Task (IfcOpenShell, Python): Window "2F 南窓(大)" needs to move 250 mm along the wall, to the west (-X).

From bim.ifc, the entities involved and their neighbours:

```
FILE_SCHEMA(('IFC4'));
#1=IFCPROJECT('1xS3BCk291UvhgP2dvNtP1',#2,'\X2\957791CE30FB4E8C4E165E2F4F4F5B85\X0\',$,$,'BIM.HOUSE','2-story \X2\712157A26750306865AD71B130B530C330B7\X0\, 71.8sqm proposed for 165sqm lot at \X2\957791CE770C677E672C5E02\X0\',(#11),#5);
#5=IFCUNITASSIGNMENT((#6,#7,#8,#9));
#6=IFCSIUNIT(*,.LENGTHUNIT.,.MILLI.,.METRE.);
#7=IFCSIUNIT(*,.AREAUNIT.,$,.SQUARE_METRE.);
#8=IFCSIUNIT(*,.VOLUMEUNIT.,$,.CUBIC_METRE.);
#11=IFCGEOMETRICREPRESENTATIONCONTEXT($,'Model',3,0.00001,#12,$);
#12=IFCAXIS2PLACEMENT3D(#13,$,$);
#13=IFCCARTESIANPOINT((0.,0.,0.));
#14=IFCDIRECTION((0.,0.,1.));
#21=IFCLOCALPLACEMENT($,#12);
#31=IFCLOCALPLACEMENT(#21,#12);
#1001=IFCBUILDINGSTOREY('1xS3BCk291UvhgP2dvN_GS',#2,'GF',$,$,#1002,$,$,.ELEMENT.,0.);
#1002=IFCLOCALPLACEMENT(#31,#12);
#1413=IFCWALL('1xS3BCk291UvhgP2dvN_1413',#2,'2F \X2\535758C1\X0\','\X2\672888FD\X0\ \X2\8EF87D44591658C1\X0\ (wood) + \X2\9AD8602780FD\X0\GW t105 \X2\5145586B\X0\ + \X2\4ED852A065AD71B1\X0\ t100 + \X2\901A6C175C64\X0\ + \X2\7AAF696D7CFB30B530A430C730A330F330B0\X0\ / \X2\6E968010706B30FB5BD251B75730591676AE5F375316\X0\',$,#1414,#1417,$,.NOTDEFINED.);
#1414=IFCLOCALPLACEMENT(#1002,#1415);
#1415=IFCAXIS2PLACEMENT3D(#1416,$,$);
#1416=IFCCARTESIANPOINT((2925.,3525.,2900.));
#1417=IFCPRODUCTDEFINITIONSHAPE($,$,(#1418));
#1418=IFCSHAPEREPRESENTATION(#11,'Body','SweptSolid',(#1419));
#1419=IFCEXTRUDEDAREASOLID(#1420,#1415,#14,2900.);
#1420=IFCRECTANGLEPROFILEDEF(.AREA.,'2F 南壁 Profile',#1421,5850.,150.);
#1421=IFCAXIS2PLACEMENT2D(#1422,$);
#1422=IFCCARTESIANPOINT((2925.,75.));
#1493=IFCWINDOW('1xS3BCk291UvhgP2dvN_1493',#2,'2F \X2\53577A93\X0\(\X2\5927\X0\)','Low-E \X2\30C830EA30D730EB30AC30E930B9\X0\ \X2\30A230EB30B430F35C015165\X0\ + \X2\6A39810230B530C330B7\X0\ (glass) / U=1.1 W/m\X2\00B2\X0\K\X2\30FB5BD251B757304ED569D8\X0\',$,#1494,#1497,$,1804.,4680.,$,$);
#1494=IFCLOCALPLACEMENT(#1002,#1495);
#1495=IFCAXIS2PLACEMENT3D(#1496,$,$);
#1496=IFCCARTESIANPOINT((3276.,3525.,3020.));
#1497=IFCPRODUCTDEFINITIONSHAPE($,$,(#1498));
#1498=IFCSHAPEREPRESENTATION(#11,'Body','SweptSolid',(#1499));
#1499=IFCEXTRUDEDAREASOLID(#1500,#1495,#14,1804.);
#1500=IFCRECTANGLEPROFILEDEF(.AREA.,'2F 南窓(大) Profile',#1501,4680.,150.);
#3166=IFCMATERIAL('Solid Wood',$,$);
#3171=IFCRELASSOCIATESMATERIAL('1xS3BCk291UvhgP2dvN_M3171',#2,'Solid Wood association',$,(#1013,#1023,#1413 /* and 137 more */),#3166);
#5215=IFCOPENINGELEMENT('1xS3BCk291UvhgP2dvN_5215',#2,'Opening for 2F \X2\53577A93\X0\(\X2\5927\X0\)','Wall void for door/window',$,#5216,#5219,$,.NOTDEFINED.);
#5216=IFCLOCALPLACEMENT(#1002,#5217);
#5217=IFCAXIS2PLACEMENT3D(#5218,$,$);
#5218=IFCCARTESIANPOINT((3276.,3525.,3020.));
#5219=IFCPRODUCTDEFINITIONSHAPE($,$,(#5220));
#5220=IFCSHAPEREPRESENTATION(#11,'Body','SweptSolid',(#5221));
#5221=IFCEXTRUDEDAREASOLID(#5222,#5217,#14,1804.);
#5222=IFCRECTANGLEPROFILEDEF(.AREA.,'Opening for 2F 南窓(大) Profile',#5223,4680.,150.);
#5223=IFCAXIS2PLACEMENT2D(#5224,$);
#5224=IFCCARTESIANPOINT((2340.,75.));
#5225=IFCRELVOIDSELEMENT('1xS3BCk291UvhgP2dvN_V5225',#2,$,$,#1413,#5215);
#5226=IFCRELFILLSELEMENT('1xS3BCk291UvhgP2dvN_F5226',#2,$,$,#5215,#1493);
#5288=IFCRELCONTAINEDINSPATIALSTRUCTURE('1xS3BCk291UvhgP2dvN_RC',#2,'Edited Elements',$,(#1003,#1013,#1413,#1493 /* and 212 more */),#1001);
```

```python
import ifcopenshell
import ifcopenshell.api.geometry
import ifcopenshell.util.placement
import ifcopenshell.util.unit

model = ifcopenshell.open("bim.ifc")
unit_scale = ifcopenshell.util.unit.calculate_unit_scale(model)

window = model.by_guid("1xS3BCk291UvhgP2dvN_1493")
opening = window.FillsVoids[0].RelatingOpeningElement
wall = opening.VoidsElements[0].RelatingBuildingElement

wall_matrix = ifcopenshell.util.placement.get_local_placement(wall.ObjectPlacement)
shift = wall_matrix[:3, 0] * -0.25 / unit_scale
before = ifcopenshell.util.placement.get_local_placement(window.ObjectPlacement)[:3, 3].copy()

# The window is not placed relative to its opening, so move both.
for product in (opening, window):
    matrix = ifcopenshell.util.placement.get_local_placement(product.ObjectPlacement)
    matrix[:3, 3] += shift
    ifcopenshell.api.geometry.edit_object_placement(model, product=product, matrix=matrix, is_si=False)

after = ifcopenshell.util.placement.get_local_placement(window.ObjectPlacement)[:3, 3]
print("window moved by", (after - before).round(3) + 0.0)

model.write("bim_updated.ifc")
```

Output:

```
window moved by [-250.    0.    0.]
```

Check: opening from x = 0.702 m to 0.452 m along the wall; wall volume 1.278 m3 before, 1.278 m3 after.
